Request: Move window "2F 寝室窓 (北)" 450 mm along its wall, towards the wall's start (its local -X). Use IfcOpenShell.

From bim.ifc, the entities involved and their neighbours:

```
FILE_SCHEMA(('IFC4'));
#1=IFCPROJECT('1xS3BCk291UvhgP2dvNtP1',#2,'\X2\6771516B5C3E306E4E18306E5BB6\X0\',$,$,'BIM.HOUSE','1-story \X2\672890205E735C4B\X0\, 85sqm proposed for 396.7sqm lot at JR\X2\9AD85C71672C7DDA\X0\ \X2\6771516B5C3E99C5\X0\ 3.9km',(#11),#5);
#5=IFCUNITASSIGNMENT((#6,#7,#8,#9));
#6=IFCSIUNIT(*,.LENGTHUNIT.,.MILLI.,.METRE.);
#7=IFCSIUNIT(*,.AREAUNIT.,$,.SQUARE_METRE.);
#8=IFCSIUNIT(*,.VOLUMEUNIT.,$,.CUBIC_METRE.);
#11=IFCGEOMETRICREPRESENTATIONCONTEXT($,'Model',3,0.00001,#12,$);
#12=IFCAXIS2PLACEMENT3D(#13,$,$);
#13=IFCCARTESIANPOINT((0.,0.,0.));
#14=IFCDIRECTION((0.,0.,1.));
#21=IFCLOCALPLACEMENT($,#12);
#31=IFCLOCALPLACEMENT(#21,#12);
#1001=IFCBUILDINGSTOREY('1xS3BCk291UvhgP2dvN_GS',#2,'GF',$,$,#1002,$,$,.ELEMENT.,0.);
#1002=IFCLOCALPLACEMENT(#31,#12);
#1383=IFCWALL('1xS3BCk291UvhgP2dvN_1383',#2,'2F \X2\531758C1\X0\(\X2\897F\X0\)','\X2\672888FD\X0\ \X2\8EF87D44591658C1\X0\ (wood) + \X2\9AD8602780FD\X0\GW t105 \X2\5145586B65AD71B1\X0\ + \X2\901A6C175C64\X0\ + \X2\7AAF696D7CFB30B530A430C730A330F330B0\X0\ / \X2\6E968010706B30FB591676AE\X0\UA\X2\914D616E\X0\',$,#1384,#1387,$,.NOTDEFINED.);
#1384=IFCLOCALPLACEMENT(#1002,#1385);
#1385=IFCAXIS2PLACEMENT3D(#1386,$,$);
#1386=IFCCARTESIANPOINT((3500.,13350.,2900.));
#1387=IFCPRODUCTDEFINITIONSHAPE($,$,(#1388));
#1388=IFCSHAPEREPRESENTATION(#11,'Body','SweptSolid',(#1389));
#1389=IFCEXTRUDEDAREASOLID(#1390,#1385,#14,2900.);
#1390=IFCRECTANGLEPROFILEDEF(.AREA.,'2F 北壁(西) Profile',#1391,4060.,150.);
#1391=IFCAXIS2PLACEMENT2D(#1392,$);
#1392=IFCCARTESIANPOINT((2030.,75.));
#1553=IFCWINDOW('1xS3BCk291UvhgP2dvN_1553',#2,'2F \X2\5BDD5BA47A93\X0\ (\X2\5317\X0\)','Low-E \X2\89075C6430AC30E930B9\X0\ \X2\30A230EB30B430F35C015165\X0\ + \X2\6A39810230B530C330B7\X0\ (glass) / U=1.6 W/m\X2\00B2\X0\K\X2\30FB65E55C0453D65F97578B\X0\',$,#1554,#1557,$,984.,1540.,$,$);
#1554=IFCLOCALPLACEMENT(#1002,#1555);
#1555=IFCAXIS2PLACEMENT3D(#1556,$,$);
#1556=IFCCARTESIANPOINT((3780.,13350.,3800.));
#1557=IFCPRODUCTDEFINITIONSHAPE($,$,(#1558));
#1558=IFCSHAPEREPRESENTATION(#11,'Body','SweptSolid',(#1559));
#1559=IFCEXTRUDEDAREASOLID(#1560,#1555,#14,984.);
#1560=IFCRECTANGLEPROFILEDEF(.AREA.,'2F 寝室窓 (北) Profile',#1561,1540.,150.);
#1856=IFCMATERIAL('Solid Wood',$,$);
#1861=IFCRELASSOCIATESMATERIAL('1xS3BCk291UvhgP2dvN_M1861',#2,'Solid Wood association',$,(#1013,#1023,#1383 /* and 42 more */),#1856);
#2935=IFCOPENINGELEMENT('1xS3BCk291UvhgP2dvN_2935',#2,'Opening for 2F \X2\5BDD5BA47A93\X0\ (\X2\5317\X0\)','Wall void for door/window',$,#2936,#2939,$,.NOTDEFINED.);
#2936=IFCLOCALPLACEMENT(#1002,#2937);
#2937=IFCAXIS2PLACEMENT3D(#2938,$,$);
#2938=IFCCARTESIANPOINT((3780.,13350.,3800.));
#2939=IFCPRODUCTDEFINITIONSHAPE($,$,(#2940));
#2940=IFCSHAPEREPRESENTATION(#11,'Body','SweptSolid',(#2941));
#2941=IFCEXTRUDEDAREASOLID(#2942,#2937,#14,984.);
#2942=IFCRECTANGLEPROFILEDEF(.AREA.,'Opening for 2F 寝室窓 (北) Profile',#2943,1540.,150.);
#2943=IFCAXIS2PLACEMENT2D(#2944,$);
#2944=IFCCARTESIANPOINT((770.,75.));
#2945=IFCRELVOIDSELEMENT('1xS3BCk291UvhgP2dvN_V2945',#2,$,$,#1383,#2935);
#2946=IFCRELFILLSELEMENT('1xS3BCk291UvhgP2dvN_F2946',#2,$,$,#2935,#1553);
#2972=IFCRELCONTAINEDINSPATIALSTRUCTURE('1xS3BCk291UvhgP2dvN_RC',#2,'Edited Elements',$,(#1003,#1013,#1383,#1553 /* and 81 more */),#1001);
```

```python
import ifcopenshell
import ifcopenshell.api.geometry
import ifcopenshell.util.placement
import ifcopenshell.util.unit

model = ifcopenshell.open("bim.ifc")
unit_scale = ifcopenshell.util.unit.calculate_unit_scale(model)

window = model.by_id(1553)
opening = window.FillsVoids[0].RelatingOpeningElement
wall = opening.VoidsElements[0].RelatingBuildingElement

wall_matrix = ifcopenshell.util.placement.get_local_placement(wall.ObjectPlacement)
shift = wall_matrix[:3, 0] * -0.45 / unit_scale
before = ifcopenshell.util.placement.get_local_placement(window.ObjectPlacement)[:3, 3].copy()

# The window is not placed relative to its opening, so move both.
for product in (opening, window):
    matrix = ifcopenshell.util.placement.get_local_placement(product.ObjectPlacement)
    matrix[:3, 3] += shift
    ifcopenshell.api.geometry.edit_object_placement(model, product=product, matrix=matrix, is_si=False)

after = ifcopenshell.util.placement.get_local_placement(window.ObjectPlacement)[:3, 3]
print("window moved by", (after - before).round(3) + 0.0)

model.write("bim_updated.ifc")
```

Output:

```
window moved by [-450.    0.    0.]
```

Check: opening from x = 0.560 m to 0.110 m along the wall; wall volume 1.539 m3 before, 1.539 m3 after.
